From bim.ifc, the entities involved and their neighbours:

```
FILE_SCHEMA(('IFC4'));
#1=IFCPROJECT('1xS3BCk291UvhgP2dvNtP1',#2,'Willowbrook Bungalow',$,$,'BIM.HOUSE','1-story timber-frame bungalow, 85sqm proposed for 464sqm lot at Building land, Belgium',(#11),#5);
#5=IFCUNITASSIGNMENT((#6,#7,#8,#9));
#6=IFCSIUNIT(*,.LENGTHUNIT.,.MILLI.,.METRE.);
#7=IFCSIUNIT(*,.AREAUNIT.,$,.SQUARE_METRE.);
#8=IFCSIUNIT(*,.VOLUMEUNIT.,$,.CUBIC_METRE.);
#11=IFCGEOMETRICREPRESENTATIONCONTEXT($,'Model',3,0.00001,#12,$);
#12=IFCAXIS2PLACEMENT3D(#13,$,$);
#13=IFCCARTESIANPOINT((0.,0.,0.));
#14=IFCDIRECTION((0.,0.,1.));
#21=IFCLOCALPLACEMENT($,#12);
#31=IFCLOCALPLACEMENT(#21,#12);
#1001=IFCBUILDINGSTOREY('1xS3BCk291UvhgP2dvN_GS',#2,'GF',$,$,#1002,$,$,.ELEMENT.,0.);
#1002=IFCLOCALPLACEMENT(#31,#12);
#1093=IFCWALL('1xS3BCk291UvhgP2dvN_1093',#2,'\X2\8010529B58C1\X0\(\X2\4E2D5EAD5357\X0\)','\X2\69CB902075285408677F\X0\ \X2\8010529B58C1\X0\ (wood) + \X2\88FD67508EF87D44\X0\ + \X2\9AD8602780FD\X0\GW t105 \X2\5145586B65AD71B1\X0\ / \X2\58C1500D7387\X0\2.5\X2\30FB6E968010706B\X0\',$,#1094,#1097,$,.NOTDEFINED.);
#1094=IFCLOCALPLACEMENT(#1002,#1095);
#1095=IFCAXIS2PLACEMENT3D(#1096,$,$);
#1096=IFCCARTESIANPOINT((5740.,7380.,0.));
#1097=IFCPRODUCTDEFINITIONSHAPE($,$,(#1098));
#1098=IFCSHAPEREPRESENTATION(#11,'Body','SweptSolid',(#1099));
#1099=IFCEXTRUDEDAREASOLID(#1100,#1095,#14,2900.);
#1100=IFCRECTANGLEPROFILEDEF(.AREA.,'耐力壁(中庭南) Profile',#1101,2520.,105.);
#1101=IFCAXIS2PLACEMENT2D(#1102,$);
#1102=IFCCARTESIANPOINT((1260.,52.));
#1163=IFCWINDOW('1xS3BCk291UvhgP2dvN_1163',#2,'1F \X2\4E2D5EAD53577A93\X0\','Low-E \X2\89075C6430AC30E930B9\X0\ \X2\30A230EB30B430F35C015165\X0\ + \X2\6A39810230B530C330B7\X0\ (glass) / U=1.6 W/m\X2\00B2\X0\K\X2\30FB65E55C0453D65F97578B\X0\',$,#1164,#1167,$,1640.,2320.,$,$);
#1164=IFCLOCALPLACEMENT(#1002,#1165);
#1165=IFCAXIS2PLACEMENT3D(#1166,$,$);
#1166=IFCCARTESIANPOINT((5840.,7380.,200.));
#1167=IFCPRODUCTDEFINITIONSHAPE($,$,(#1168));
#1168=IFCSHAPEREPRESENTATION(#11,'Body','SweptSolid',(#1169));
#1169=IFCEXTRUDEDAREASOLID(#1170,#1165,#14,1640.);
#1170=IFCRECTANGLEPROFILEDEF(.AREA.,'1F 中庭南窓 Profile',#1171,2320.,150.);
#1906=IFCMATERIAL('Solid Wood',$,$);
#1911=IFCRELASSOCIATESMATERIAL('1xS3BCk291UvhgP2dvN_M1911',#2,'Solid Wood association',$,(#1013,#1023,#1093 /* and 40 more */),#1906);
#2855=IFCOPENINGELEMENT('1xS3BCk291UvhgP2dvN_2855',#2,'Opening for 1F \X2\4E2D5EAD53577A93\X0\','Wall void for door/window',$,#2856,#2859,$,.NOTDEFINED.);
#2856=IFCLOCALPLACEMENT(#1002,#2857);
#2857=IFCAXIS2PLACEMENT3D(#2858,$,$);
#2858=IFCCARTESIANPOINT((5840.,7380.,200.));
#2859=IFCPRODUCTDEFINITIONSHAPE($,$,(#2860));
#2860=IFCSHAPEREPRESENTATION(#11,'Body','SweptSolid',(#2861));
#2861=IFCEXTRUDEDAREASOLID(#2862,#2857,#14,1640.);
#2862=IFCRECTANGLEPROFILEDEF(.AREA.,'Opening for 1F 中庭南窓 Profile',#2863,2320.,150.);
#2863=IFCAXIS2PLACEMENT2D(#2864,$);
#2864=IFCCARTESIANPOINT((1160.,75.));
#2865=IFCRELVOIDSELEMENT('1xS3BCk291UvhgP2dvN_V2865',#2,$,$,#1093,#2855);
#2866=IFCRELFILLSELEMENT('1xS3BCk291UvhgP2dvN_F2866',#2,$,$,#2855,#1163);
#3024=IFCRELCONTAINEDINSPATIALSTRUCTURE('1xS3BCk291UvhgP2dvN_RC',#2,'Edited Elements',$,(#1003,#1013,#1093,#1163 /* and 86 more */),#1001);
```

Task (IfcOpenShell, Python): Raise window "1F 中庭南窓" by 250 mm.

```python
import numpy as np
import ifcopenshell
import ifcopenshell.api.geometry
import ifcopenshell.util.placement
import ifcopenshell.util.unit

model = ifcopenshell.open("bim.ifc")
unit_scale = ifcopenshell.util.unit.calculate_unit_scale(model)

window = model.by_guid("1xS3BCk291UvhgP2dvN_1163")
opening = window.FillsVoids[0].RelatingOpeningElement
dz = 0.25 / unit_scale

shift = np.array([0.0, 0.0, dz])
# The window is not placed relative to its opening, so move both.
for product in (opening, window):
    matrix = ifcopenshell.util.placement.get_local_placement(product.ObjectPlacement)
    matrix[:3, 3] += shift
    ifcopenshell.api.geometry.edit_object_placement(model, product=product, matrix=matrix, is_si=False)

print(f"moved by {dz * unit_scale:+.3f} m")

model.write("bim_updated.ifc")
```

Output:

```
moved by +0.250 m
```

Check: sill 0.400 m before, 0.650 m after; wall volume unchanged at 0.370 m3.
